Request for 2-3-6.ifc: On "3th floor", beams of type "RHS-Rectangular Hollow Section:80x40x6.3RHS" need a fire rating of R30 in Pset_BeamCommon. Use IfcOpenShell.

First a look at what the model holds.

```python
import ifcopenshell
import ifcopenshell.util.element

model = ifcopenshell.open("2-3-6.ifc")
print(model.schema)
storey = next(s for s in model.by_type("IfcBuildingStorey") if s.Name == "3th floor")
beams = [e for e in ifcopenshell.util.element.get_decomposition(storey) if e.is_a("IfcBeam")]
seen = {}
for e in beams:
    element_type = ifcopenshell.util.element.get_type(e)
    key = (element_type.Name if element_type != e and element_type else None, ifcopenshell.util.element.get_pset(e, "Pset_BeamCommon", "FireRating"))
    seen[key] = seen.get(key, 0) + 1
for (name, value), count in sorted(seen.items(), key=str):
    print(count, "x", name, "|", value)
```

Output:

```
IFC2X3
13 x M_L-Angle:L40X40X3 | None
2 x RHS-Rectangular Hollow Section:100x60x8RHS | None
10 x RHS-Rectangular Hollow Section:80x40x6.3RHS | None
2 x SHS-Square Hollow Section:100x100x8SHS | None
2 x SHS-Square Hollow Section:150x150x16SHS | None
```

```python
import ifcopenshell
import ifcopenshell.api.pset
import ifcopenshell.util.element

model = ifcopenshell.open("2-3-6.ifc")

storey = next(s for s in model.by_type("IfcBuildingStorey") if s.Name == "3th floor")
beams = [e for e in ifcopenshell.util.element.get_decomposition(storey) if e.is_a("IfcBeam")]

count = 0
for e in beams:
    element_type = ifcopenshell.util.element.get_type(e)
    if element_type in (None, e) or element_type.Name != "RHS-Rectangular Hollow Section:80x40x6.3RHS":
        continue
    # add_pset returns the element's existing set when there is one.
    pset = ifcopenshell.api.pset.add_pset(model, product=e, name="Pset_BeamCommon")
    ifcopenshell.api.pset.edit_pset(model, pset=pset, properties={"FireRating": "R30"})
    count += 1

print(count, "beams updated")

model.write("2-3-6-out.ifc")
```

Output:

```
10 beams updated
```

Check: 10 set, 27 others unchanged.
